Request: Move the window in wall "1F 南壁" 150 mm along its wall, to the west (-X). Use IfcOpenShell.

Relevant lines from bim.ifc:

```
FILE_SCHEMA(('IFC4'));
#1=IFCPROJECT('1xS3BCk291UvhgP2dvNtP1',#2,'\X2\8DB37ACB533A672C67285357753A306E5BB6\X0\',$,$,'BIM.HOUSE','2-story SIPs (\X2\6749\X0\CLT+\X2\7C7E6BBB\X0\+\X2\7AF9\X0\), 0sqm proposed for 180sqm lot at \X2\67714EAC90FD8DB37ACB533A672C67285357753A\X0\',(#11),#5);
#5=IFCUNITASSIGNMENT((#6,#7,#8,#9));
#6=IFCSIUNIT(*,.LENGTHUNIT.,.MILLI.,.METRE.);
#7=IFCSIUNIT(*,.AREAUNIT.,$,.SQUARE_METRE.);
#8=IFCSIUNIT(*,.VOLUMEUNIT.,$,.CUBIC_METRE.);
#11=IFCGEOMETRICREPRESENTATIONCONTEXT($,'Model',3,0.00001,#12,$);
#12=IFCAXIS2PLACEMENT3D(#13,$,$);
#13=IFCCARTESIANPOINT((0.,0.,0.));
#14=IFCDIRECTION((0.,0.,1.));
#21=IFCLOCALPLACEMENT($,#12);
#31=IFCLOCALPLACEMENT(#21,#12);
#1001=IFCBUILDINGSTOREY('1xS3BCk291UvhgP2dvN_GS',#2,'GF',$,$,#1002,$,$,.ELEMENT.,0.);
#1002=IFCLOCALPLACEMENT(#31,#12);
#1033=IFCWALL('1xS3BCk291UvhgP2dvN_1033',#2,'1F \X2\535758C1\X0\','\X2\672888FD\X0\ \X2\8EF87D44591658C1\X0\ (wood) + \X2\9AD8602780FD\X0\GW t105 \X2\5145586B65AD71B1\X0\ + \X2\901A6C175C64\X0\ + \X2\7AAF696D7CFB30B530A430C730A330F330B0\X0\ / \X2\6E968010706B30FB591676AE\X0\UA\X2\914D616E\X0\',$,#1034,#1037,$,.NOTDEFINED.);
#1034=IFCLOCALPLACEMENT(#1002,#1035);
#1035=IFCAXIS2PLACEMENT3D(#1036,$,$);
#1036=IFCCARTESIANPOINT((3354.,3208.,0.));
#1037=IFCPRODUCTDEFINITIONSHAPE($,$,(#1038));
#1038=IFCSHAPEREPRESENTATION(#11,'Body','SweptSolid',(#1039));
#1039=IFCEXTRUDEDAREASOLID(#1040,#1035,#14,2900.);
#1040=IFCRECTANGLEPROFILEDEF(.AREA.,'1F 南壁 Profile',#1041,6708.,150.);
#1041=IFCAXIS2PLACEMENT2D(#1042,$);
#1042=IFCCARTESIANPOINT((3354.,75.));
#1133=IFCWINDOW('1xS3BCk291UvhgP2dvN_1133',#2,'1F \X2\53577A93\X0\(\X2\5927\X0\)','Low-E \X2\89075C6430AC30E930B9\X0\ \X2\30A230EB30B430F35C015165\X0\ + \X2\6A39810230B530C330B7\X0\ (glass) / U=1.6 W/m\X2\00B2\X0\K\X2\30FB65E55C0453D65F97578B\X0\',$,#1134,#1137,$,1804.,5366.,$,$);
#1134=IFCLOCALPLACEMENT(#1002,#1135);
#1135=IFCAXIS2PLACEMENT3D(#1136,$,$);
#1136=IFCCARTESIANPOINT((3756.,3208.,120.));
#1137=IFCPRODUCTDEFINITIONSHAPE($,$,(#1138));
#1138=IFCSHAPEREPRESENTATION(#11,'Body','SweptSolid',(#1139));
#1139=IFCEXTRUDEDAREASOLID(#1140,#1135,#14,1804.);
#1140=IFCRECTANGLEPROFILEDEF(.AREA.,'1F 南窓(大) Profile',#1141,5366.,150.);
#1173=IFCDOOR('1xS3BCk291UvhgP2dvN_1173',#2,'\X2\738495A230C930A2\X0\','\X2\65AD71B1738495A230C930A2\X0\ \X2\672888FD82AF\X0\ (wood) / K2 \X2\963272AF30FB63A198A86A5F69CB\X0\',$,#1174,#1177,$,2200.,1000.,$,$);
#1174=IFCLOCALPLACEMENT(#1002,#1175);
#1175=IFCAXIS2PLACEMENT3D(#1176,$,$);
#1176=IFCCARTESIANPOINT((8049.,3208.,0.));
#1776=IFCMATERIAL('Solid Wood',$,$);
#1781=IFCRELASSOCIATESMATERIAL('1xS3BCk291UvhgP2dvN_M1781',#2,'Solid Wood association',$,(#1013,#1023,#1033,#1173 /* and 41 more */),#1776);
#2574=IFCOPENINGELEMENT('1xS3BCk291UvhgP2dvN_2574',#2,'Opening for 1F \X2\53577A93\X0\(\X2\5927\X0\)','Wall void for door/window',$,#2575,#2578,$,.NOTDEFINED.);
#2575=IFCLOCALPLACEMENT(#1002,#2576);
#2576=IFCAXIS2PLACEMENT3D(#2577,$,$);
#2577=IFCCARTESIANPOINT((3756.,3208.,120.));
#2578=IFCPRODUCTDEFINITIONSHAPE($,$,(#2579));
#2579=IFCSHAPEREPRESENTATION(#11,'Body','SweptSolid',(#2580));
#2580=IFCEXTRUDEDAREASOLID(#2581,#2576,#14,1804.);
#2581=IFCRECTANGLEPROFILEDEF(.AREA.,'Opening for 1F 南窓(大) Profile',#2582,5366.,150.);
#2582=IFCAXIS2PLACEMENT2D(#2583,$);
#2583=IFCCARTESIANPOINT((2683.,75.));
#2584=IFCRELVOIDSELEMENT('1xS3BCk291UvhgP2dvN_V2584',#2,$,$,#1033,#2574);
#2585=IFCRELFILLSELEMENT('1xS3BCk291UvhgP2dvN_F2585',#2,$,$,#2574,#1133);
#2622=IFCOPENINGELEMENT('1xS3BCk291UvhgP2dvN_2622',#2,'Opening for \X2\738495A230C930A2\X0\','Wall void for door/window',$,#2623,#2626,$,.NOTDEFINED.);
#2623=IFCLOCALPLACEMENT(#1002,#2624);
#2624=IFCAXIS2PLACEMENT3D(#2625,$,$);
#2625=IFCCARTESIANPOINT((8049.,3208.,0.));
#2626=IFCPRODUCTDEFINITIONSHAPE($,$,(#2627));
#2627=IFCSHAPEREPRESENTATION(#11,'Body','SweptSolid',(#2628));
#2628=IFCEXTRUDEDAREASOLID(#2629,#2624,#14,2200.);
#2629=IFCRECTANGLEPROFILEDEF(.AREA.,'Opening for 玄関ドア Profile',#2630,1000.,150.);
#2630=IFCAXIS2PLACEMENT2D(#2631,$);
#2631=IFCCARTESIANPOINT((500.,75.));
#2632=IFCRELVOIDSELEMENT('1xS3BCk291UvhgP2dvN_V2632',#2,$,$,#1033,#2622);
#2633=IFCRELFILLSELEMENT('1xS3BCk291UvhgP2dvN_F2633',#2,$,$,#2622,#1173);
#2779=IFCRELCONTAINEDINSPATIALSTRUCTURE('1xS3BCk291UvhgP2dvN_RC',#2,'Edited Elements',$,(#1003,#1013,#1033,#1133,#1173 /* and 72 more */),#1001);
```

```python
import ifcopenshell
import ifcopenshell.api.geometry
import ifcopenshell.util.placement
import ifcopenshell.util.unit

model = ifcopenshell.open("bim.ifc")
unit_scale = ifcopenshell.util.unit.calculate_unit_scale(model)

window = model.by_guid("1xS3BCk291UvhgP2dvN_1133")
opening = window.FillsVoids[0].RelatingOpeningElement
wall = opening.VoidsElements[0].RelatingBuildingElement

wall_matrix = ifcopenshell.util.placement.get_local_placement(wall.ObjectPlacement)
shift = wall_matrix[:3, 0] * -0.15 / unit_scale
before = ifcopenshell.util.placement.get_local_placement(window.ObjectPlacement)[:3, 3].copy()

# The window is not placed relative to its opening, so move both.
for product in (opening, window):
    matrix = ifcopenshell.util.placement.get_local_placement(product.ObjectPlacement)
    matrix[:3, 3] += shift
    ifcopenshell.api.geometry.edit_object_placement(model, product=product, matrix=matrix, is_si=False)

after = ifcopenshell.util.placement.get_local_placement(window.ObjectPlacement)[:3, 3]
print("window moved by", (after - before).round(3) + 0.0)

model.write("bim-out.ifc")
```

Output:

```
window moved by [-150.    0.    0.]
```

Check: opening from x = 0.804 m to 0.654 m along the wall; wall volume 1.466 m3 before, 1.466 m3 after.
